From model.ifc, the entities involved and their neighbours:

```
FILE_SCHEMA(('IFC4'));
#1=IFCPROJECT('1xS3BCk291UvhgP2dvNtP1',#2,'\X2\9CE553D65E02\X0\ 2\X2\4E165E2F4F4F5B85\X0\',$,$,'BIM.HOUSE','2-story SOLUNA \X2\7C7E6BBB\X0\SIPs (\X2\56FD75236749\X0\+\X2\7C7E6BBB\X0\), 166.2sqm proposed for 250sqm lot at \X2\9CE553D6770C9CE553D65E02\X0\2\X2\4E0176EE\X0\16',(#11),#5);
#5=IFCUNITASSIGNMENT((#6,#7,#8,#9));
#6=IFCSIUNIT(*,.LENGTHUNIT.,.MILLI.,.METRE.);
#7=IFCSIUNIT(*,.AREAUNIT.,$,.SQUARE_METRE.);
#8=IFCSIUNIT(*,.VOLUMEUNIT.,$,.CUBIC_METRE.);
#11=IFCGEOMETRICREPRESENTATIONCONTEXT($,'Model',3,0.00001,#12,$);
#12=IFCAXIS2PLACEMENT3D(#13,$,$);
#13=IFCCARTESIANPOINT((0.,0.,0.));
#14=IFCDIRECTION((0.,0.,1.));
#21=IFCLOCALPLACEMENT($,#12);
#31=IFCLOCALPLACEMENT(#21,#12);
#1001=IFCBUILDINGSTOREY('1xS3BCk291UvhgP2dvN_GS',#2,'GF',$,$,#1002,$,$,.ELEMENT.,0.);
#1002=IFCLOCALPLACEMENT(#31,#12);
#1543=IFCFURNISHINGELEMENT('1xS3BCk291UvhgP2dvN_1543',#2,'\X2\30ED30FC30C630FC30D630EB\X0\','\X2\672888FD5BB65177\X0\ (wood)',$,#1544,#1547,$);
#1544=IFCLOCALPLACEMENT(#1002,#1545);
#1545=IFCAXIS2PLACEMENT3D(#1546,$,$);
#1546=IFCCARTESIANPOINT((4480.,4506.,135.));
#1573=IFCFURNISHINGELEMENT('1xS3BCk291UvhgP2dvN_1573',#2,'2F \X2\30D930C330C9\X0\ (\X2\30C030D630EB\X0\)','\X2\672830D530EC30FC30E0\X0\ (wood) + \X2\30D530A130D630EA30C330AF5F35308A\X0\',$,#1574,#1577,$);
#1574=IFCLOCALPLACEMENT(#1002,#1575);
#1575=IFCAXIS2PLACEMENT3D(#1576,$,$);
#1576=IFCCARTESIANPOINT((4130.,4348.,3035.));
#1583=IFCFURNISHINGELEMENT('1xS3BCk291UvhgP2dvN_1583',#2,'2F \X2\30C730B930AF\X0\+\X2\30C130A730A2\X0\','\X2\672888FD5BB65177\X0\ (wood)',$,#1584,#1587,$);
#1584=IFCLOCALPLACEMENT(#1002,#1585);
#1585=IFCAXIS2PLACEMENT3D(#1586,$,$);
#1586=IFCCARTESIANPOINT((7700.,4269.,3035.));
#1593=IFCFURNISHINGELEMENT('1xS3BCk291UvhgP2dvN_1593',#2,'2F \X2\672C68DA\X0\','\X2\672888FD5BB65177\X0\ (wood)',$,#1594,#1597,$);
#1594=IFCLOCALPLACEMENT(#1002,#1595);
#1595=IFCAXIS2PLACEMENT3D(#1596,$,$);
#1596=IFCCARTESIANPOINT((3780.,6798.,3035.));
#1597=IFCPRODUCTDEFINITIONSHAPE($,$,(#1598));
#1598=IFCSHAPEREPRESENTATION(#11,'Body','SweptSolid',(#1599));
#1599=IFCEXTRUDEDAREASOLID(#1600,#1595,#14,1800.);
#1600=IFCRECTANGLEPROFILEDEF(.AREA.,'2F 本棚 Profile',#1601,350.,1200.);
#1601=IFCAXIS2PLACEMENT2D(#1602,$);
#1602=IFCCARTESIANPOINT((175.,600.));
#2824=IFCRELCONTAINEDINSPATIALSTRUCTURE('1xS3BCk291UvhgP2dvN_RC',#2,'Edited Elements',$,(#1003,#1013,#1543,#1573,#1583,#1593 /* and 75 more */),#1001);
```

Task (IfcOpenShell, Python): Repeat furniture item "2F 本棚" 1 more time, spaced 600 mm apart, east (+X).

```python
import numpy as np
import ifcopenshell
import ifcopenshell.api.geometry
import ifcopenshell.api.root
import ifcopenshell.util.element
import ifcopenshell.util.placement
import ifcopenshell.util.unit

model = ifcopenshell.open("model.ifc")
unit_scale = ifcopenshell.util.unit.calculate_unit_scale(model)


def reuse_history(source, copy):
    """copy_class also copies each property set's owner history, people and application; keep the originals."""
    for rel in copy.IsDefinedBy:
        if rel.is_a("IfcRelDefinesByProperties") and (history := rel.RelatingPropertyDefinition.OwnerHistory):
            rel.RelatingPropertyDefinition.OwnerHistory = source.OwnerHistory
            ifcopenshell.util.element.remove_deep2(model, history)


source = model.by_guid("1xS3BCk291UvhgP2dvN_1593")
base = ifcopenshell.util.placement.get_local_placement(source.ObjectPlacement)
step = np.array([1.0, 0.0, 0.0]) * 0.6 / unit_scale

for i in range(1, 2):
    copy = ifcopenshell.api.root.copy_class(model, product=source)
    copy.Representation = ifcopenshell.util.element.copy_deep(
        model, source.Representation, exclude=["IfcGeometricRepresentationContext", "IfcRepresentationMap"]
    )
    reuse_history(source, copy)
    matrix = base.copy()
    matrix[:3, 3] += i * step
    print("added at", matrix[:3, 3].round(3) + 0.0)
    ifcopenshell.api.geometry.edit_object_placement(model, product=copy, matrix=matrix, is_si=False)

model.write("model_v2.ifc")
```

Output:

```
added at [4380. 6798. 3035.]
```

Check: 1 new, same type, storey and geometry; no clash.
